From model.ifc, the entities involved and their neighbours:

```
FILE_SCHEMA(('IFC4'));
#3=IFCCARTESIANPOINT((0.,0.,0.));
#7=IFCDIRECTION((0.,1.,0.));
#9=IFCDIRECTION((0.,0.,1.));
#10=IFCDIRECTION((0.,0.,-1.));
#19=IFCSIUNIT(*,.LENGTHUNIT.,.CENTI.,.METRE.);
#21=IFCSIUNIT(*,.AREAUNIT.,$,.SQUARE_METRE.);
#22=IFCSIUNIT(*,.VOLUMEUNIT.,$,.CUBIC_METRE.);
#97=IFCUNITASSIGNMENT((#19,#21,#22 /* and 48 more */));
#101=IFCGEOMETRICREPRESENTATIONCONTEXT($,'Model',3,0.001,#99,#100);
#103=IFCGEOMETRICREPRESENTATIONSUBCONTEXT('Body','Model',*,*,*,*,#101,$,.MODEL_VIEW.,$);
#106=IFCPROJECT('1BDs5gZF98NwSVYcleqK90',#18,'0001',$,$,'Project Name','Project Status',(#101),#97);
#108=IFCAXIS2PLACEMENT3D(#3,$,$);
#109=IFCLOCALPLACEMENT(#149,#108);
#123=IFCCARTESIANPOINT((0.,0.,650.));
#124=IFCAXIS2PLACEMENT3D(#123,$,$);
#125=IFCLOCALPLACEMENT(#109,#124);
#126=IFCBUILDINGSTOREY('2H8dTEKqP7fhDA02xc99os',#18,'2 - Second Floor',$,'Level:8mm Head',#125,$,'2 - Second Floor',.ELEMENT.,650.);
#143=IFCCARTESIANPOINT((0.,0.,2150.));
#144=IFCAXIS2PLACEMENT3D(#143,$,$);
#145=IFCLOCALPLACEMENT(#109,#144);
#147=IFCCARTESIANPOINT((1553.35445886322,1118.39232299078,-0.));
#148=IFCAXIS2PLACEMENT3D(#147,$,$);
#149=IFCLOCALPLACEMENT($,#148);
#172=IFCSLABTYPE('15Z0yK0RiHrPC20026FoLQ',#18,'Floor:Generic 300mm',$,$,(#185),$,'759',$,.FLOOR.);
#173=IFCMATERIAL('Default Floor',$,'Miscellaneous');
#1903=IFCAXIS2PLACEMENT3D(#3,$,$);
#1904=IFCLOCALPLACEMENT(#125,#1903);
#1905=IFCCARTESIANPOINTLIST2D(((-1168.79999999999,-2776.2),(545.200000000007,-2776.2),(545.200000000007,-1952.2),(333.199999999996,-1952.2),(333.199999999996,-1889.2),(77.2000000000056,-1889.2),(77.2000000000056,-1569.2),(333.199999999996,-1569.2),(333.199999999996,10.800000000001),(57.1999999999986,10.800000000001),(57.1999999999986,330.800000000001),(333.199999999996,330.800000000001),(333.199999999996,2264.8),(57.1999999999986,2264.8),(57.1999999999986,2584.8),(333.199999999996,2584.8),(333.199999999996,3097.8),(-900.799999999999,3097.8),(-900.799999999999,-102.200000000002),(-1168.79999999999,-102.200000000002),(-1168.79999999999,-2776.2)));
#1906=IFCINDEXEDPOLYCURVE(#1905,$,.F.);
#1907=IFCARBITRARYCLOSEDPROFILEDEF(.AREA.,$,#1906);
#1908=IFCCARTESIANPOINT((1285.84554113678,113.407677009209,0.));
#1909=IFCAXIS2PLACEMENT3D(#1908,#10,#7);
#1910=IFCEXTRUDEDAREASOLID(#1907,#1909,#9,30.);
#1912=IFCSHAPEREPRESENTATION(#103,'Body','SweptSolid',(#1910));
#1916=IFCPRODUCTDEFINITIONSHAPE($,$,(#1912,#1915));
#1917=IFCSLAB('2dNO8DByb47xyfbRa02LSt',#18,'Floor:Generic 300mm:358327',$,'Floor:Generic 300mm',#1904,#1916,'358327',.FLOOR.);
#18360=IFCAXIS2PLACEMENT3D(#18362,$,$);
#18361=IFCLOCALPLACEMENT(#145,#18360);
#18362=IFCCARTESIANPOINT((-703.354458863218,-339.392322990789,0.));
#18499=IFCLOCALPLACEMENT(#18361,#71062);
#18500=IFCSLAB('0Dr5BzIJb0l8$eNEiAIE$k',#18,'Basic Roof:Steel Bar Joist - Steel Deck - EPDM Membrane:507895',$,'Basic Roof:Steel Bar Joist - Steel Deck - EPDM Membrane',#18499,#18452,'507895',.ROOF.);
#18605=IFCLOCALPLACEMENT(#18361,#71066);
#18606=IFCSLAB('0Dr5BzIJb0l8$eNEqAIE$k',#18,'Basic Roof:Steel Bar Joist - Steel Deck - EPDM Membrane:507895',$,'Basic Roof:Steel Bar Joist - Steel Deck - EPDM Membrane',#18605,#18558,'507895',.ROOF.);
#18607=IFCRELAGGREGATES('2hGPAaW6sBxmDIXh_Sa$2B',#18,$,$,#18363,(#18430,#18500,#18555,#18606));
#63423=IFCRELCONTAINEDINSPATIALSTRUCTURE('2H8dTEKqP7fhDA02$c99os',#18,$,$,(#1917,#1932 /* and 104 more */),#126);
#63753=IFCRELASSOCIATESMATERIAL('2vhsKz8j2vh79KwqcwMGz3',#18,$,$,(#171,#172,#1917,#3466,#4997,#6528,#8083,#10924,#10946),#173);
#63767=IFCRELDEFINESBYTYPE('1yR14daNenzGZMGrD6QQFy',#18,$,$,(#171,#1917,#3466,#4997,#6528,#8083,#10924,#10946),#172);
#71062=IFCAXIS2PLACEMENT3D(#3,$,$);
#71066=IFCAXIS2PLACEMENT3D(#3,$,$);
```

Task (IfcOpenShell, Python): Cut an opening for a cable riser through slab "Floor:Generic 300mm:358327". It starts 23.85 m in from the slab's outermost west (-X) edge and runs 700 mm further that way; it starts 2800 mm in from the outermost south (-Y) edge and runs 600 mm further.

```python
import numpy as np
import ifcopenshell
import ifcopenshell.api.feature
import ifcopenshell.api.geometry
import ifcopenshell.api.root
import ifcopenshell.geom
import ifcopenshell.util.placement
import ifcopenshell.util.representation
import ifcopenshell.util.shape
import ifcopenshell.util.unit

model = ifcopenshell.open("model.ifc")
unit_scale = ifcopenshell.util.unit.calculate_unit_scale(model)
settings = ifcopenshell.geom.settings()


def volume(element):
    """Net volume in cubic metres, openings subtracted."""
    shape = ifcopenshell.geom.create_shape(settings, element)
    return ifcopenshell.util.shape.get_volume(shape.geometry)


slab = model.by_guid("2dNO8DByb47xyfbRa02LSt")
before = volume(slab)

# Extent in the slab's own axes, in metres. The edges named are its -X and -Y sides.
slab_shape = ifcopenshell.geom.create_shape(settings, slab)
vertices = ifcopenshell.util.shape.get_vertices(slab_shape.geometry)
x_min, y_min, bottom = vertices.min(axis=0)
top = vertices[:, 2].max()

opening = ifcopenshell.api.root.create_entity(model, ifc_class="IfcOpeningElement", name="Cable riser opening", predefined_type="OPENING")
context = ifcopenshell.util.representation.get_context(model, "Model", "Body", "MODEL_VIEW")
width, depth = 0.7, 0.6
outline = [(0.0, 0.0), (width, 0.0), (width, depth), (0.0, depth), (0.0, 0.0)]
# Overshoot both faces by 50 mm so the cut is clean.
shape = ifcopenshell.api.geometry.add_slab_representation(
    model, context=context, depth=top - bottom + 0.1, polyline=outline
)
ifcopenshell.api.geometry.assign_representation(model, product=opening, representation=shape)

matrix = ifcopenshell.util.placement.get_local_placement(slab.ObjectPlacement)
matrix[:, 3] = matrix @ np.append(np.array([x_min + 23.85, y_min + 2.8, bottom - 0.05]) / unit_scale, 1.0)
ifcopenshell.api.geometry.edit_object_placement(model, product=opening, matrix=matrix, is_si=False)
ifcopenshell.api.feature.add_feature(model, feature=opening, element=slab)

after = volume(slab)

print(f"slab volume {before:.3f} -> {after:.3f} m3")

model.write("model-out.ifc")
```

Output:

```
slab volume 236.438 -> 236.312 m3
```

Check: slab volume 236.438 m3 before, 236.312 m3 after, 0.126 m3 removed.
